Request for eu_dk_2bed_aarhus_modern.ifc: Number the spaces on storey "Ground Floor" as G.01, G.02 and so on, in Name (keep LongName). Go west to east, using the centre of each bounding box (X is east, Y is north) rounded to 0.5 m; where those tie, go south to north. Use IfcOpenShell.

First a look at what the model holds.

```python
import ifcopenshell
import ifcopenshell.util.element
import ifcopenshell.util.placement

model = ifcopenshell.open("eu_dk_2bed_aarhus_modern.ifc")
print(model.schema)
storey = next(s for s in model.by_type("IfcBuildingStorey") if s.Name == "Ground Floor")
spaces = [e for e in ifcopenshell.util.element.get_decomposition(storey) if e.is_a("IfcSpace")]
for e in sorted(spaces, key=lambda e: e.id()):
    origin = ifcopenshell.util.placement.get_local_placement(e.ObjectPlacement)[:3, 3]
    print(e.id(), e.Name, e.LongName, origin.round(2) + 0.0, sep=" | ")
```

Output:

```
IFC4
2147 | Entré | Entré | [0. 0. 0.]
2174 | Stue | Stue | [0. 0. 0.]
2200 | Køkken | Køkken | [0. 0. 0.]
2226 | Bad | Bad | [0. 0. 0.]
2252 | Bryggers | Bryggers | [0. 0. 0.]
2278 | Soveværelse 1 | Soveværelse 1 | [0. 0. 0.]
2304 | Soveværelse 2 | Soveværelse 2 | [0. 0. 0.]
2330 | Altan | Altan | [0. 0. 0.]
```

```python
import ifcopenshell
import ifcopenshell.geom
import ifcopenshell.util.element
import ifcopenshell.util.shape

model = ifcopenshell.open("eu_dk_2bed_aarhus_modern.ifc")
settings = ifcopenshell.geom.settings()
settings.set("use-world-coords", True)


def centre(element):
    shape = ifcopenshell.geom.create_shape(settings, element)
    return ifcopenshell.util.shape.get_bbox_centroid(shape.geometry)


storey = next(s for s in model.by_type("IfcBuildingStorey") if s.Name == "Ground Floor")
spaces = [e for e in ifcopenshell.util.element.get_decomposition(storey) if e.is_a("IfcSpace")]

# Insertion points can sit at a corner or the storey origin, so sort by the geometry (in metres).
centres = {e: centre(e) for e in spaces}
spaces.sort(key=lambda e: (round(centres[e][0] / 0.5), centres[e][1]))

for i, e in enumerate(spaces, start=1):
    number = f"G.{i:02d}"
    e.Name = number
    print(e.id(), number)

model.write("eu_dk_2bed_aarhus_modern_updated.ifc")
```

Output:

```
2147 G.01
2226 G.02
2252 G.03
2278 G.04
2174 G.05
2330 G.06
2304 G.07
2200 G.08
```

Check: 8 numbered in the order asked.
